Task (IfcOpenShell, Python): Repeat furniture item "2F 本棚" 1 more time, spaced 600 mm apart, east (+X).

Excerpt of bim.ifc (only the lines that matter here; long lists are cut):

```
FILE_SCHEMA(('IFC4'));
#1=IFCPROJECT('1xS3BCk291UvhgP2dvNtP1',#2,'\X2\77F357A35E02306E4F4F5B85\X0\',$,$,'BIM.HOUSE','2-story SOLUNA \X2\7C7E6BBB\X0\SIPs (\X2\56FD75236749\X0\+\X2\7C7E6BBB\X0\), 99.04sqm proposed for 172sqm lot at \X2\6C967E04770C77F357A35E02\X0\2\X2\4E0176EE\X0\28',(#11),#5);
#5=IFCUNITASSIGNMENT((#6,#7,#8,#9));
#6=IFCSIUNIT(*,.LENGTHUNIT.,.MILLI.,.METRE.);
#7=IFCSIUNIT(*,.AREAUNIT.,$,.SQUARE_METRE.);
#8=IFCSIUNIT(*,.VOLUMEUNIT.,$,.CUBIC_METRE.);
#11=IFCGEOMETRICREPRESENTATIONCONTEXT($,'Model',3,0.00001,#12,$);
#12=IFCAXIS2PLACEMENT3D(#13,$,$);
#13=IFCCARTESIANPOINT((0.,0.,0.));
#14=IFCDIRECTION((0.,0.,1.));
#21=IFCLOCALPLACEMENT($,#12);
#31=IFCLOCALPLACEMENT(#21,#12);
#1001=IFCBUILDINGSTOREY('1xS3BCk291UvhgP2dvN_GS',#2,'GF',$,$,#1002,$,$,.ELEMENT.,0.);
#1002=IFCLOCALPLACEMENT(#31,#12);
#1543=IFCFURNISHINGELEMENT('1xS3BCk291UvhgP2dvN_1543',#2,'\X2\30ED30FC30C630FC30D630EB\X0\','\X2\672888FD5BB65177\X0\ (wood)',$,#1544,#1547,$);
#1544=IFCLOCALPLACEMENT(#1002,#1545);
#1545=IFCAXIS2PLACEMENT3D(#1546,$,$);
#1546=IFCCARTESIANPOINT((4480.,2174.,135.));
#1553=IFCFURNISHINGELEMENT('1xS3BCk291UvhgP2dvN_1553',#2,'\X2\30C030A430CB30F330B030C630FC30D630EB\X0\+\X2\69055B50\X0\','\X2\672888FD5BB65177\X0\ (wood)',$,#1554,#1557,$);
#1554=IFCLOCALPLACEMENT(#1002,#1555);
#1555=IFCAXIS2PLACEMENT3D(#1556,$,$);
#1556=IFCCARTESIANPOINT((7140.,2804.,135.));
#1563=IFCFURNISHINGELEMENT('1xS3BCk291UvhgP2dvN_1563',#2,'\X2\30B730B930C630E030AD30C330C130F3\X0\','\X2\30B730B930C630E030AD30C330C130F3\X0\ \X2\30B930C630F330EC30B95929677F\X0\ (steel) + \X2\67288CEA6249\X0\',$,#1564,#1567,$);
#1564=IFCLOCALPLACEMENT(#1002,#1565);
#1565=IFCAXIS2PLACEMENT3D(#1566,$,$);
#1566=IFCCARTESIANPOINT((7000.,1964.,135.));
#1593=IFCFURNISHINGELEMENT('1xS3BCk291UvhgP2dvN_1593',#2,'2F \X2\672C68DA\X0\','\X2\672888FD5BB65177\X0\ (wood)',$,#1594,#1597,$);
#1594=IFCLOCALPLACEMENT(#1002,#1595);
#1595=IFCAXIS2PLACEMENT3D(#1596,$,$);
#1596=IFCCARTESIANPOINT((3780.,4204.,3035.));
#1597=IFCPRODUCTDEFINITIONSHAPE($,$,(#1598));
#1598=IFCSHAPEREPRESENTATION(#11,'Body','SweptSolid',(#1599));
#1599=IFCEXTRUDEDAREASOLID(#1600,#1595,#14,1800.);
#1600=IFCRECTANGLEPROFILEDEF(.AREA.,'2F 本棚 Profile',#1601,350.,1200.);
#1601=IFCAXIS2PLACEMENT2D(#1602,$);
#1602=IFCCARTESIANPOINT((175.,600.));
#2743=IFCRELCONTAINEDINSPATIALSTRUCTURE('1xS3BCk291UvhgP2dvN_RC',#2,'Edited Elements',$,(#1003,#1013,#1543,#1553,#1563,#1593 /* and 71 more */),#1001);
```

```python
import numpy as np
import ifcopenshell
import ifcopenshell.api.geometry
import ifcopenshell.api.root
import ifcopenshell.util.element
import ifcopenshell.util.placement

model = ifcopenshell.open("bim.ifc")


def reuse_history(source, copy):
    """copy_class also copies each property set's owner history, people and application; keep the originals."""
    for rel in copy.IsDefinedBy:
        if rel.is_a("IfcRelDefinesByProperties") and (history := rel.RelatingPropertyDefinition.OwnerHistory):
            rel.RelatingPropertyDefinition.OwnerHistory = source.OwnerHistory
            ifcopenshell.util.element.remove_deep2(model, history)


source = model.by_guid("1xS3BCk291UvhgP2dvN_1593")
base = ifcopenshell.util.placement.get_local_placement(source.ObjectPlacement)
step = np.array([1.0, 0.0, 0.0]) * 600.0

for i in range(1, 2):
    copy = ifcopenshell.api.root.copy_class(model, product=source)
    copy.Representation = ifcopenshell.util.element.copy_deep(
        model, source.Representation, exclude=["IfcGeometricRepresentationContext", "IfcRepresentationMap"]
    )
    reuse_history(source, copy)
    matrix = base.copy()
    matrix[:3, 3] += i * step
    print("added at", matrix[:3, 3].round(3) + 0.0)
    ifcopenshell.api.geometry.edit_object_placement(model, product=copy, matrix=matrix, is_si=False)

model.write("bim_rev.ifc")
```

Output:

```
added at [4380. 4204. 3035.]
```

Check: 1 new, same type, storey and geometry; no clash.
